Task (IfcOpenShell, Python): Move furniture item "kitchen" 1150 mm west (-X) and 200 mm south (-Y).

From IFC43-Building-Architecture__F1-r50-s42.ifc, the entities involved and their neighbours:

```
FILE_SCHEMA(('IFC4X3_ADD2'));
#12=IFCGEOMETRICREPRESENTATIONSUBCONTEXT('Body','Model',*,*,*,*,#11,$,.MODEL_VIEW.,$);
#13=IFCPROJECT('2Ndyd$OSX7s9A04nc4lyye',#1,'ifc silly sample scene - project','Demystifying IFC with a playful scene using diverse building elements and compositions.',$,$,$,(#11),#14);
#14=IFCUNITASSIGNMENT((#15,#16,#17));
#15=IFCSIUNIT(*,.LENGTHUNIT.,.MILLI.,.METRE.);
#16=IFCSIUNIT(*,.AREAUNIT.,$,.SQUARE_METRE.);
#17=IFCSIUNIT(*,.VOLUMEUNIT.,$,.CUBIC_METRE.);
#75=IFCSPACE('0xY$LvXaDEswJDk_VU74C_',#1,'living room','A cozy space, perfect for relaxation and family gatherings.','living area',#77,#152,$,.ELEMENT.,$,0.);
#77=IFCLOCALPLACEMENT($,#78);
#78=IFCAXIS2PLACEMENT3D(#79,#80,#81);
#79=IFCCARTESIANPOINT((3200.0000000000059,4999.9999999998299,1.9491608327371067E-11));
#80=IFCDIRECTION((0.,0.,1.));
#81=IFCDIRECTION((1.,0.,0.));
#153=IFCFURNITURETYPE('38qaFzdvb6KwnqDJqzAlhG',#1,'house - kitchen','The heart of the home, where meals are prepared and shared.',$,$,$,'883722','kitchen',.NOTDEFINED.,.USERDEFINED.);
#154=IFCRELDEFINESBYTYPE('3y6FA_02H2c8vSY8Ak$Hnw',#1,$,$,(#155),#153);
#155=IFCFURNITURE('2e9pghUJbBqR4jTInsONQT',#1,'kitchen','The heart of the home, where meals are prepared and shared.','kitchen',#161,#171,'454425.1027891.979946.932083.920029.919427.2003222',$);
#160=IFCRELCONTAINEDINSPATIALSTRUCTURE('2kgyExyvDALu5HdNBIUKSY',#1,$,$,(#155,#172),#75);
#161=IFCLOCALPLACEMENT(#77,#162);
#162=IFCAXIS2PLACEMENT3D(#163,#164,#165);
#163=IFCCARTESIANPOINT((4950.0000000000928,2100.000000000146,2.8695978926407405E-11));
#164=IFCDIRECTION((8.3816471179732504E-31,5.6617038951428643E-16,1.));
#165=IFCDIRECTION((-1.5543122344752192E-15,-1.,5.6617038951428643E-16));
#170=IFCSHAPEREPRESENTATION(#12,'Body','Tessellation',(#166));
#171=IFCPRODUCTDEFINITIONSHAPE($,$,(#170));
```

```python
import ifcopenshell
import ifcopenshell.api.geometry
import ifcopenshell.util.placement

model = ifcopenshell.open("IFC43-Building-Architecture__F1-r50-s42.ifc")

item = model.by_guid("2e9pghUJbBqR4jTInsONQT")
matrix = ifcopenshell.util.placement.get_local_placement(item.ObjectPlacement)
matrix[0, 3] -= 1150.0
matrix[1, 3] -= 200.0
ifcopenshell.api.geometry.edit_object_placement(model, product=item, matrix=matrix, is_si=False)

print(ifcopenshell.util.placement.get_local_placement(item.ObjectPlacement).round(3) + 0.0)

model.write("IFC43-Building-Architecture__F1-r50-s42-out.ifc")
```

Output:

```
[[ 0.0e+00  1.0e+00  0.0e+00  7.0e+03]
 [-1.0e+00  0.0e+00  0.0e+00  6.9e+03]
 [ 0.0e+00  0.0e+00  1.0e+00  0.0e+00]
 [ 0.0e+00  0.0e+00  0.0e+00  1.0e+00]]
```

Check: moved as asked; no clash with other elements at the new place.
